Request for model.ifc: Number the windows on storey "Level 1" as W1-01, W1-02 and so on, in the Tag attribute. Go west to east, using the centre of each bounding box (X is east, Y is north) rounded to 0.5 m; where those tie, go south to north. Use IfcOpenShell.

First a look at what the model holds.

```python
import ifcopenshell
import ifcopenshell.util.element
import ifcopenshell.util.placement

model = ifcopenshell.open("model.ifc")
print(model.schema)
storey = next(s for s in model.by_type("IfcBuildingStorey") if s.Name == "Level 1")
windows = [e for e in ifcopenshell.util.element.get_decomposition(storey) if e.is_a("IfcWindow")]
for e in sorted(windows, key=lambda e: e.id()):
    origin = ifcopenshell.util.placement.get_local_placement(e.ObjectPlacement)[:3, 3]
    print(e.id(), e.Tag, e.Name, origin.round(2) + 0.0, sep=" | ")
```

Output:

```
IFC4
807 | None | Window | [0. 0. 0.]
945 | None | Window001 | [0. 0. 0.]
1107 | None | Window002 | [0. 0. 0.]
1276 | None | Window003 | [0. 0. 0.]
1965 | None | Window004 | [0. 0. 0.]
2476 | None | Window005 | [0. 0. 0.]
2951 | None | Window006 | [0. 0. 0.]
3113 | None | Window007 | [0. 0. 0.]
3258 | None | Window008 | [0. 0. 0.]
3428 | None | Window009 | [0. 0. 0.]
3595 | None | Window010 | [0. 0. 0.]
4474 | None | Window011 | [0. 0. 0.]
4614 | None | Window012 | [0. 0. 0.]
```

```python
import ifcopenshell
import ifcopenshell.geom
import ifcopenshell.util.element
import ifcopenshell.util.shape

model = ifcopenshell.open("model.ifc")
settings = ifcopenshell.geom.settings()
settings.set("use-world-coords", True)


def centre(element):
    shape = ifcopenshell.geom.create_shape(settings, element)
    return ifcopenshell.util.shape.get_bbox_centroid(shape.geometry)


storey = next(s for s in model.by_type("IfcBuildingStorey") if s.Name == "Level 1")
windows = [e for e in ifcopenshell.util.element.get_decomposition(storey) if e.is_a("IfcWindow")]

# Insertion points can sit at a corner or the storey origin, so sort by the geometry (in metres).
centres = {e: centre(e) for e in windows}
windows.sort(key=lambda e: (round(centres[e][0] / 0.5), centres[e][1]))

for i, e in enumerate(windows, start=1):
    number = f"W1-{i:02d}"
    e.Tag = number
    print(e.id(), number)

model.write("model_rev.ifc")
```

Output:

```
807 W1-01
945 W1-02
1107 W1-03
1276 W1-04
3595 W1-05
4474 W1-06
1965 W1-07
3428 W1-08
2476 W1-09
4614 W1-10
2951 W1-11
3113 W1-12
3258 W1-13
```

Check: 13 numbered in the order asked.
